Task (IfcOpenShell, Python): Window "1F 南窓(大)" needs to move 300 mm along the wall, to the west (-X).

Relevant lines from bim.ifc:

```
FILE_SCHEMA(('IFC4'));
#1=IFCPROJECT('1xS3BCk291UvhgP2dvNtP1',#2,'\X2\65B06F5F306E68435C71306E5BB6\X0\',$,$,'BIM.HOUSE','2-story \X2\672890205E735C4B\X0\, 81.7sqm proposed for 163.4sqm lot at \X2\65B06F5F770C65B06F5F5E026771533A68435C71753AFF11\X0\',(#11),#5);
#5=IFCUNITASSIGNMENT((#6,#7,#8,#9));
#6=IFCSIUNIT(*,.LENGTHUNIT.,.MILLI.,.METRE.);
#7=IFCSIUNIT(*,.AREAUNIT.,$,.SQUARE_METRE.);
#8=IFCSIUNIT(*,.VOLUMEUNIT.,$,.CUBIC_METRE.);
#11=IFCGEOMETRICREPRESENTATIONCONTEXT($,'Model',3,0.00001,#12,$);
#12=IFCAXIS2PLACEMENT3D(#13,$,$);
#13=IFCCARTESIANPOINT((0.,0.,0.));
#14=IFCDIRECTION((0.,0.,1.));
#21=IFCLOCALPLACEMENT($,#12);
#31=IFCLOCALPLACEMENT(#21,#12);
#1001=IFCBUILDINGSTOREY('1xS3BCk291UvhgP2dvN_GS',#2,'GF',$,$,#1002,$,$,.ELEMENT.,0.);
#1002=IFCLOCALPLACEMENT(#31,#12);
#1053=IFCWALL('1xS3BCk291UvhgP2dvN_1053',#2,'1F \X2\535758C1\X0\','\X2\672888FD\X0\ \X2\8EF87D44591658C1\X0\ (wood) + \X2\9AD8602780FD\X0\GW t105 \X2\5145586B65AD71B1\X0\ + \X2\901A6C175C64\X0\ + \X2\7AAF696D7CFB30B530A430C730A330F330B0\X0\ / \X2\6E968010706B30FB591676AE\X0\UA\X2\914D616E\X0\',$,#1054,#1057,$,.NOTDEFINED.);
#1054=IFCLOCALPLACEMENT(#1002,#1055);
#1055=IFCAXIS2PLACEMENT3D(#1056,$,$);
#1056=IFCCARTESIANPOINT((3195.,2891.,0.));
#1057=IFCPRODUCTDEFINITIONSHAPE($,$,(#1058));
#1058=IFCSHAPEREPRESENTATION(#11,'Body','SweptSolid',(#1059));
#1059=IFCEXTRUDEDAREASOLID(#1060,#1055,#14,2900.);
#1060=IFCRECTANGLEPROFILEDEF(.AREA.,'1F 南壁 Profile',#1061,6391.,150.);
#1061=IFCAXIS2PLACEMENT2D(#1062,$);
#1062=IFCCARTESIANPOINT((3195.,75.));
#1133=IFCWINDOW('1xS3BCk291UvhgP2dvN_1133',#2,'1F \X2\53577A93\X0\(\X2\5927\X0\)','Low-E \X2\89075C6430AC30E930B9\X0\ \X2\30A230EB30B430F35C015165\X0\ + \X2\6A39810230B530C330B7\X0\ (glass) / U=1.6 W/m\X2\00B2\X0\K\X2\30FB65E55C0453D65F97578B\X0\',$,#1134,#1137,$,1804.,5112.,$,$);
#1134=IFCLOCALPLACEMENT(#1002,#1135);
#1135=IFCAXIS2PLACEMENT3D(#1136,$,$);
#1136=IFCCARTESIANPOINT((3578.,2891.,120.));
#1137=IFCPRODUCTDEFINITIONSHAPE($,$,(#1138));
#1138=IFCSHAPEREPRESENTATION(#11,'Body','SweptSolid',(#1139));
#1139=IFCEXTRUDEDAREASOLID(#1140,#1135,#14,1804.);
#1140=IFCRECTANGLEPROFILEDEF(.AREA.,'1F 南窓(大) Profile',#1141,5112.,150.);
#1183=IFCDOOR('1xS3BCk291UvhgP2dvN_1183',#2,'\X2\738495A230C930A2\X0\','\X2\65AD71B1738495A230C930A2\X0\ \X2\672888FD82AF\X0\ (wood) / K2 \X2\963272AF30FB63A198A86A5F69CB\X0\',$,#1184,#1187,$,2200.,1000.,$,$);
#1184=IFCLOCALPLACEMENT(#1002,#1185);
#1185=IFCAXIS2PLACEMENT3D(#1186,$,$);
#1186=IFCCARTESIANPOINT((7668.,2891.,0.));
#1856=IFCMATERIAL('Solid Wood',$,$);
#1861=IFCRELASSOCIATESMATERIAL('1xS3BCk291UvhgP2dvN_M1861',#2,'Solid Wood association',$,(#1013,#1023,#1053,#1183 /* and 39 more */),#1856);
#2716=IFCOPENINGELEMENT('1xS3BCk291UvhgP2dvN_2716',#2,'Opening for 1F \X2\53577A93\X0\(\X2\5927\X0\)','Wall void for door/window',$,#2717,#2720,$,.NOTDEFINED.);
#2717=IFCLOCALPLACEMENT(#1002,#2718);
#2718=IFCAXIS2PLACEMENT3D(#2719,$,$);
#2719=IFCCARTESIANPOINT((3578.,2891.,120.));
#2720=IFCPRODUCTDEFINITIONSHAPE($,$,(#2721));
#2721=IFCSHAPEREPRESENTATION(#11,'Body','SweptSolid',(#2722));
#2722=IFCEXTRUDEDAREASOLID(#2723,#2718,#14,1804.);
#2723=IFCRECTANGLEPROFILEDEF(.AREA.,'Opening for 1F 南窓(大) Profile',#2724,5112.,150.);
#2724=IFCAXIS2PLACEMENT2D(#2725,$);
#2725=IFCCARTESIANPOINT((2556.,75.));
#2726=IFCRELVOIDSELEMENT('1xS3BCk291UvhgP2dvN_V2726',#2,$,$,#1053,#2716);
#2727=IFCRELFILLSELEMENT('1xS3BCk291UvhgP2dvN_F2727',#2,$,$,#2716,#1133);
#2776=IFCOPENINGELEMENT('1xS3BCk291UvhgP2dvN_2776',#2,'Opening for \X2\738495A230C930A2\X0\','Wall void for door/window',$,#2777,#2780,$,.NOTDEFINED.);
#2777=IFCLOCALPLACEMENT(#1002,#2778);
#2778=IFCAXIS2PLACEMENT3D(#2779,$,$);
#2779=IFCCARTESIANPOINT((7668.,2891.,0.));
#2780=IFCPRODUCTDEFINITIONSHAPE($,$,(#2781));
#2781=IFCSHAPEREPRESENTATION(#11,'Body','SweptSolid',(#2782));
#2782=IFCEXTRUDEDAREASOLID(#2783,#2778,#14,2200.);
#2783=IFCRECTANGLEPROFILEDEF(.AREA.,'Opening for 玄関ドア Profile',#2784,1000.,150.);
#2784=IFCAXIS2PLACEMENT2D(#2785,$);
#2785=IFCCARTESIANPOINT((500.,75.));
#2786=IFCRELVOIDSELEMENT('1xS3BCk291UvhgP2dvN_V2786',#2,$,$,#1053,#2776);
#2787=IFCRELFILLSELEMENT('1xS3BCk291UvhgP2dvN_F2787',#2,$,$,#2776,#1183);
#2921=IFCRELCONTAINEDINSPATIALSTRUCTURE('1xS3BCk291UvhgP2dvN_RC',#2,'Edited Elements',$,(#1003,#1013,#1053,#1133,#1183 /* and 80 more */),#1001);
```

```python
import ifcopenshell
import ifcopenshell.api.geometry
import ifcopenshell.util.placement
import ifcopenshell.util.unit

model = ifcopenshell.open("bim.ifc")
unit_scale = ifcopenshell.util.unit.calculate_unit_scale(model)

window = model.by_id(1133)
opening = window.FillsVoids[0].RelatingOpeningElement
wall = opening.VoidsElements[0].RelatingBuildingElement

wall_matrix = ifcopenshell.util.placement.get_local_placement(wall.ObjectPlacement)
shift = wall_matrix[:3, 0] * -0.3 / unit_scale
before = ifcopenshell.util.placement.get_local_placement(window.ObjectPlacement)[:3, 3].copy()

# The window is not placed relative to its opening, so move both.
for product in (opening, window):
    matrix = ifcopenshell.util.placement.get_local_placement(product.ObjectPlacement)
    matrix[:3, 3] += shift
    ifcopenshell.api.geometry.edit_object_placement(model, product=product, matrix=matrix, is_si=False)

after = ifcopenshell.util.placement.get_local_placement(window.ObjectPlacement)[:3, 3]
print("window moved by", (after - before).round(3) + 0.0)

model.write("bim_rev.ifc")
```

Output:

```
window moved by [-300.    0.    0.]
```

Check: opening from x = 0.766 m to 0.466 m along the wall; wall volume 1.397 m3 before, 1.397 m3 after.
